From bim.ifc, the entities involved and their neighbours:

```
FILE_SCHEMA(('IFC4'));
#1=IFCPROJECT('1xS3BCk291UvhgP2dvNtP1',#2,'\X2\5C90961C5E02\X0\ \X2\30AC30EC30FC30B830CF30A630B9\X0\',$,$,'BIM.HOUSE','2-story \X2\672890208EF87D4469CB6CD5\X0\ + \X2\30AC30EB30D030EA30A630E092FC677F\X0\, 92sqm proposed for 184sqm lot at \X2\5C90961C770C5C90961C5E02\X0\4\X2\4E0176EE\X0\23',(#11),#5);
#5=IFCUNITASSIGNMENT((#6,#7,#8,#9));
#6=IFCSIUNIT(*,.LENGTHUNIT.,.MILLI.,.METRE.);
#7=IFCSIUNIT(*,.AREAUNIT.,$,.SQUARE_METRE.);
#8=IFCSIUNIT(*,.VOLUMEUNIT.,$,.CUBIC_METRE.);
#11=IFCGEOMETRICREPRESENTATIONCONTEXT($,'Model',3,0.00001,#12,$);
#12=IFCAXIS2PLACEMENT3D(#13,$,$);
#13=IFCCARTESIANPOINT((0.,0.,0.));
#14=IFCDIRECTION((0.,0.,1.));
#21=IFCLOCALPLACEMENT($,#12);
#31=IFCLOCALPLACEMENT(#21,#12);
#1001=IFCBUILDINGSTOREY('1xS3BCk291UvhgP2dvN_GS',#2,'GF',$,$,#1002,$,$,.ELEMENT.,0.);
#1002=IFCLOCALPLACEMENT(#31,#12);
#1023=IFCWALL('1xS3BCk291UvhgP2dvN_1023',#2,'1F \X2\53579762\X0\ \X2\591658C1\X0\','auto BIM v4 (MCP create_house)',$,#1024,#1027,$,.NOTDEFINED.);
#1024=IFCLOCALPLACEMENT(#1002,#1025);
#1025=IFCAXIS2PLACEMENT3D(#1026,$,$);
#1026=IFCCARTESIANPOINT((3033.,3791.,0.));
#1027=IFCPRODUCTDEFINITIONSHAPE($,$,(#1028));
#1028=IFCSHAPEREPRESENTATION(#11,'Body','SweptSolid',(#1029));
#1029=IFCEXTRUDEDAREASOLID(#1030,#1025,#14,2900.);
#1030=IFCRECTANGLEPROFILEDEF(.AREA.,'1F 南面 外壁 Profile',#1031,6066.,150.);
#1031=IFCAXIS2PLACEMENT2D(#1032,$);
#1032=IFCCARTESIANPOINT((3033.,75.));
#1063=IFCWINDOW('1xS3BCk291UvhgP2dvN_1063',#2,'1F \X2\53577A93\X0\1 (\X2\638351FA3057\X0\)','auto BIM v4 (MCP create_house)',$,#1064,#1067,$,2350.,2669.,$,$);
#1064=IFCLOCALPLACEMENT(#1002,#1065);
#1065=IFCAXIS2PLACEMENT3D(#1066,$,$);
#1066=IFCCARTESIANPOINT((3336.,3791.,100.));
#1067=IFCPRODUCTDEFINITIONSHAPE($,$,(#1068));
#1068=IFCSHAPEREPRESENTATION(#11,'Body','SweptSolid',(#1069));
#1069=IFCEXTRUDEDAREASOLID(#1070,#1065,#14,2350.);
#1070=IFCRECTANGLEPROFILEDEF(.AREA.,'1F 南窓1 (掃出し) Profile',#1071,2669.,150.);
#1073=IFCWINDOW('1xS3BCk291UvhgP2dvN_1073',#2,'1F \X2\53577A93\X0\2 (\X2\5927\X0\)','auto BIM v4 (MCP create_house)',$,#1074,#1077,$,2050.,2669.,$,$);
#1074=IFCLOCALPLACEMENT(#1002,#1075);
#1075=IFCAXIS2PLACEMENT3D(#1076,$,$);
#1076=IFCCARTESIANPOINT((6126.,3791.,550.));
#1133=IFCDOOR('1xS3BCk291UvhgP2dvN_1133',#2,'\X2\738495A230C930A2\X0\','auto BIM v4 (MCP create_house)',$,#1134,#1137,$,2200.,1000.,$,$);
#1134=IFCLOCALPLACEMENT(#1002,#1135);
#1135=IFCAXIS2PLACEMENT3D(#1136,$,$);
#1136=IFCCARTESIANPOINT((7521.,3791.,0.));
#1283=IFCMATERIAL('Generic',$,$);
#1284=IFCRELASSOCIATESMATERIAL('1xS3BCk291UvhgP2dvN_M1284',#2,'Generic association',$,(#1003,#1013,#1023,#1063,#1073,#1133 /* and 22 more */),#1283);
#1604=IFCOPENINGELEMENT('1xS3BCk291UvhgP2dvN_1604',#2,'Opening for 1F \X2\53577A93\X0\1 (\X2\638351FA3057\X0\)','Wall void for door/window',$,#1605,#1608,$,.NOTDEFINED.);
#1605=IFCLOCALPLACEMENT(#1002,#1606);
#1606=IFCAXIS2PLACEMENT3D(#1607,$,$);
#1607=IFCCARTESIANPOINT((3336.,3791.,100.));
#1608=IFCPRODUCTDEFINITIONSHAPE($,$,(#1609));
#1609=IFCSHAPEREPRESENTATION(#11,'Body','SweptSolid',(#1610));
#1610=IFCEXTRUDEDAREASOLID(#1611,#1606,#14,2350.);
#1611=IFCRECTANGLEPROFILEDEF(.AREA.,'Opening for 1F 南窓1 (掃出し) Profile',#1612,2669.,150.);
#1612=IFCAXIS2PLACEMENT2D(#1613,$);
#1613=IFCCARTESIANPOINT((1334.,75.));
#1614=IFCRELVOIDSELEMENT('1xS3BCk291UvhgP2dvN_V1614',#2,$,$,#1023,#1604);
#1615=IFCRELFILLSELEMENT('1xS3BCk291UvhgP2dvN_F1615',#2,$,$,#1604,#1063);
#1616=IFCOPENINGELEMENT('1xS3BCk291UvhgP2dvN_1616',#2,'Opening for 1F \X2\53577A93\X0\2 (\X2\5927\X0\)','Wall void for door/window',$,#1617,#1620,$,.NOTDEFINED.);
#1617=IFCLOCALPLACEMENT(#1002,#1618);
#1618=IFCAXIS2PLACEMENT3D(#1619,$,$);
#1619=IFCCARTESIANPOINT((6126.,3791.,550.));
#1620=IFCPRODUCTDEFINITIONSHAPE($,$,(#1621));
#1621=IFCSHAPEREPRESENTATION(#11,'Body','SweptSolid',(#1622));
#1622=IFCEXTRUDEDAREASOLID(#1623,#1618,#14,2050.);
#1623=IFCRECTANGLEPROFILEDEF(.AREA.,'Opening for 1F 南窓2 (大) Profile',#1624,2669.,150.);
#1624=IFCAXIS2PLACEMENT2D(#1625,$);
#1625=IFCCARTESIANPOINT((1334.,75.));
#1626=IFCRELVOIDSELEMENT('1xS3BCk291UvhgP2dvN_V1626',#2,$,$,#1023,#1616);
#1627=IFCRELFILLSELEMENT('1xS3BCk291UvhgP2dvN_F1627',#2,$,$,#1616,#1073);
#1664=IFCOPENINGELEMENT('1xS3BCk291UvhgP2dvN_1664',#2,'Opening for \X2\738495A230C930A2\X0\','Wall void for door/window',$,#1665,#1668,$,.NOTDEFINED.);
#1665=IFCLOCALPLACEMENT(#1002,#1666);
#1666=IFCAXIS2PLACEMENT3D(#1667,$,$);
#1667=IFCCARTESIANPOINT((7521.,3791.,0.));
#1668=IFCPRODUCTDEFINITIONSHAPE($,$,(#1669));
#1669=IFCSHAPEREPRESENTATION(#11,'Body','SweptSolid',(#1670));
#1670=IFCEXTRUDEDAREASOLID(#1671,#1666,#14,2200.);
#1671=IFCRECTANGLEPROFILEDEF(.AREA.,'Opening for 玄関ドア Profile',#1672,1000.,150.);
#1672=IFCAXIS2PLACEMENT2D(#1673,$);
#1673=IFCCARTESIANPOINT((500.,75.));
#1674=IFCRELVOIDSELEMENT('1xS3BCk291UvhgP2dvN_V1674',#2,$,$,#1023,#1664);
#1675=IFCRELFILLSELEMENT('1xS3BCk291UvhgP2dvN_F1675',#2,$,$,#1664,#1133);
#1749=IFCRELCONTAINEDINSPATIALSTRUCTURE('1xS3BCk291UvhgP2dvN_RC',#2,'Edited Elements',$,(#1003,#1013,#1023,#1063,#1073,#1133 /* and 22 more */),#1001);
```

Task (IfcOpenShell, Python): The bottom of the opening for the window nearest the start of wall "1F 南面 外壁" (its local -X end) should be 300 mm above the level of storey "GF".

```python
import numpy as np
import ifcopenshell
import ifcopenshell.api.geometry
import ifcopenshell.geom
import ifcopenshell.util.element
import ifcopenshell.util.placement
import ifcopenshell.util.shape
import ifcopenshell.util.unit

model = ifcopenshell.open("bim.ifc")
unit_scale = ifcopenshell.util.unit.calculate_unit_scale(model)

window = model.by_guid("1xS3BCk291UvhgP2dvN_1063")
opening = window.FillsVoids[0].RelatingOpeningElement
storey = ifcopenshell.util.element.get_container(window, ifc_class="IfcBuildingStorey")
level = ifcopenshell.util.placement.get_local_placement(storey.ObjectPlacement)[2, 3]

# The opening's origin need not be at the sill, so measure its lowest point.
shape = ifcopenshell.geom.create_shape(ifcopenshell.geom.settings(), opening)
bottom = ifcopenshell.util.shape.get_shape_bottom_elevation(shape, shape.geometry) / unit_scale
dz = level + 0.3 / unit_scale - bottom

shift = np.array([0.0, 0.0, dz])
# The window is not placed relative to its opening, so move both.
for product in (opening, window):
    matrix = ifcopenshell.util.placement.get_local_placement(product.ObjectPlacement)
    matrix[:3, 3] += shift
    ifcopenshell.api.geometry.edit_object_placement(model, product=product, matrix=matrix, is_si=False)

print(f"moved by {dz * unit_scale:+.3f} m")

model.write("bim_edited.ifc")
```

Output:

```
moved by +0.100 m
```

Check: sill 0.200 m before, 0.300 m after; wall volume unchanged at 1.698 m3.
